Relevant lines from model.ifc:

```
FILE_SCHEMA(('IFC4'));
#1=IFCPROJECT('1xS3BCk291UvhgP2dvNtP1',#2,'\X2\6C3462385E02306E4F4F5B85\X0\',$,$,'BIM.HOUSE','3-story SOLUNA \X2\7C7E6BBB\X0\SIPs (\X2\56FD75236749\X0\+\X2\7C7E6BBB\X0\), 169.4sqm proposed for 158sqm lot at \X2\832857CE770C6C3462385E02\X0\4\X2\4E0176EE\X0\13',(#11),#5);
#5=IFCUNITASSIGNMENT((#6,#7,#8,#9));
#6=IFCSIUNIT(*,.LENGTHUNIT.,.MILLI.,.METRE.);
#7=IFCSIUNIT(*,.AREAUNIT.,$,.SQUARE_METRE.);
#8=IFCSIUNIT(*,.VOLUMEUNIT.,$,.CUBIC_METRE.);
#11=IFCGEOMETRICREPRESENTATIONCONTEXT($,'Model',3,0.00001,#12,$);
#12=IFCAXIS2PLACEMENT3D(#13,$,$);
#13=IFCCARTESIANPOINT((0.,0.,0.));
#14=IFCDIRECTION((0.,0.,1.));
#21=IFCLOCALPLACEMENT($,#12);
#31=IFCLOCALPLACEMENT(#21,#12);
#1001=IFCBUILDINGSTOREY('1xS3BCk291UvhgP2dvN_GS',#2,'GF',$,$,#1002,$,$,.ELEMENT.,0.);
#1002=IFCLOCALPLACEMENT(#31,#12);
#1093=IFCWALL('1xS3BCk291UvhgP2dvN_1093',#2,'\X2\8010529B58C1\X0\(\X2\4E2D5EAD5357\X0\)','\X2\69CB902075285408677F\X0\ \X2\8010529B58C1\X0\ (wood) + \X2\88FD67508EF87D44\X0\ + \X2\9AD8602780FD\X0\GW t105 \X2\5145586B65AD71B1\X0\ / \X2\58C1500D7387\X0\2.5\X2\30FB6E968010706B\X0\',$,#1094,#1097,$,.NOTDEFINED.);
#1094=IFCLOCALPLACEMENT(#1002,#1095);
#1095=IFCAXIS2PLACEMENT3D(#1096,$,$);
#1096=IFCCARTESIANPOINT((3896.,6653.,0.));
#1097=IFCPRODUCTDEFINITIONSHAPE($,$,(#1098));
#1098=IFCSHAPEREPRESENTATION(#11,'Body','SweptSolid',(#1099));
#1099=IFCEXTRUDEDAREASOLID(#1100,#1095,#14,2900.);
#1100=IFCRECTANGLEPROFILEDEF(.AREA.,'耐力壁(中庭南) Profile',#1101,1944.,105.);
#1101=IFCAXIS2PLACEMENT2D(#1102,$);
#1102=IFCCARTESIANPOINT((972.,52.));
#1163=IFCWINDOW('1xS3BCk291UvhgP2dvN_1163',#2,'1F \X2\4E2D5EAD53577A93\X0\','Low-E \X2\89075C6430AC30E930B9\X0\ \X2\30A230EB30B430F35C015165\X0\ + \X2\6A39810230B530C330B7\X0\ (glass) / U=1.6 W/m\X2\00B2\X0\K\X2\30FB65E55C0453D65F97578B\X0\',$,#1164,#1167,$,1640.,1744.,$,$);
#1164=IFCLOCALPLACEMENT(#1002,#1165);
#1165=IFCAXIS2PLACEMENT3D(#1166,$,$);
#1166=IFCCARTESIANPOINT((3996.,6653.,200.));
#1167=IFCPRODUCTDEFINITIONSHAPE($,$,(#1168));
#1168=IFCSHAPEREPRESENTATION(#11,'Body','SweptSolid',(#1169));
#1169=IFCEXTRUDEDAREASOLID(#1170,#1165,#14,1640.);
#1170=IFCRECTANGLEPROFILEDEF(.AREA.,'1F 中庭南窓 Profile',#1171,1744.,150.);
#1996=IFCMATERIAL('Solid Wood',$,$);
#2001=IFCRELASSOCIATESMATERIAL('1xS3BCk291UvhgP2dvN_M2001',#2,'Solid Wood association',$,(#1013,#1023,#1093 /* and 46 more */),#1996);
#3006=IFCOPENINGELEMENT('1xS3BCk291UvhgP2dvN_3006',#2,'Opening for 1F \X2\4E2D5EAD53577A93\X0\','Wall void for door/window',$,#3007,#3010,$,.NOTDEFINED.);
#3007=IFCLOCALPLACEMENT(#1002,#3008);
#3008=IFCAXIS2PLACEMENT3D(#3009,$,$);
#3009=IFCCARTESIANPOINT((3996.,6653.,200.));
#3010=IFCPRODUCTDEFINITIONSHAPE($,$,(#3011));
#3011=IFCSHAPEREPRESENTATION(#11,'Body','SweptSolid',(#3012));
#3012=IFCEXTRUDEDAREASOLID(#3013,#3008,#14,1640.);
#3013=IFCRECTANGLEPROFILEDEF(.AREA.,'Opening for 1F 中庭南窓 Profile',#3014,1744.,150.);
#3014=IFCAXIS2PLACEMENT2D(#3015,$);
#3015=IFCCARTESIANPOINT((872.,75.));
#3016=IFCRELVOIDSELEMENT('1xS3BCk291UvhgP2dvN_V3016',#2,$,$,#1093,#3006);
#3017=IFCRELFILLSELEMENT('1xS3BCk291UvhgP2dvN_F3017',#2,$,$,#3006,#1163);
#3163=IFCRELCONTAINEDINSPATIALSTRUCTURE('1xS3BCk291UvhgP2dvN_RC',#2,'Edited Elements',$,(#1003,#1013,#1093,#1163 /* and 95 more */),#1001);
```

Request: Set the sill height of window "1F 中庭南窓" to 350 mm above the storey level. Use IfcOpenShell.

```python
import numpy as np
import ifcopenshell
import ifcopenshell.api.geometry
import ifcopenshell.geom
import ifcopenshell.util.element
import ifcopenshell.util.placement
import ifcopenshell.util.shape
import ifcopenshell.util.unit

model = ifcopenshell.open("model.ifc")
unit_scale = ifcopenshell.util.unit.calculate_unit_scale(model)

window = model.by_id(1163)
opening = window.FillsVoids[0].RelatingOpeningElement
storey = ifcopenshell.util.element.get_container(window, ifc_class="IfcBuildingStorey")
level = ifcopenshell.util.placement.get_local_placement(storey.ObjectPlacement)[2, 3]

# The opening's origin need not be at the sill, so measure its lowest point.
shape = ifcopenshell.geom.create_shape(ifcopenshell.geom.settings(), opening)
bottom = ifcopenshell.util.shape.get_shape_bottom_elevation(shape, shape.geometry) / unit_scale
dz = level + 350.0 - bottom

shift = np.array([0.0, 0.0, dz])
# The window is not placed relative to its opening, so move both.
for product in (opening, window):
    matrix = ifcopenshell.util.placement.get_local_placement(product.ObjectPlacement)
    matrix[:3, 3] += shift
    ifcopenshell.api.geometry.edit_object_placement(model, product=product, matrix=matrix, is_si=False)

print(f"moved by {dz * unit_scale:+.3f} m")

model.write("model_rev.ifc")
```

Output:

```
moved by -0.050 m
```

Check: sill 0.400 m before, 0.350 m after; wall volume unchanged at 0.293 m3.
